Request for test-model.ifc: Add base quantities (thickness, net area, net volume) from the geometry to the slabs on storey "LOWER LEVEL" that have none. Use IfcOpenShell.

First a look at what the model holds.

```python
import ifcopenshell
import ifcopenshell.util.element
import ifcopenshell.util.unit

model = ifcopenshell.open("test-model.ifc")
print(model.schema)
for unit_type in ("LENGTHUNIT", "AREAUNIT", "VOLUMEUNIT"):
    print(unit_type, ifcopenshell.util.unit.calculate_unit_scale(model, unit_type))
storey = next(s for s in model.by_type("IfcBuildingStorey") if s.Name == "LOWER LEVEL")
slabs = [e for e in ifcopenshell.util.element.get_decomposition(storey) if e.is_a("IfcSlab")]
for e in sorted(slabs, key=lambda e: e.id()):
    print(e.id(), e.is_a(), e.Name, list(ifcopenshell.util.element.get_psets(e, qtos_only=True)), sep=" | ")
```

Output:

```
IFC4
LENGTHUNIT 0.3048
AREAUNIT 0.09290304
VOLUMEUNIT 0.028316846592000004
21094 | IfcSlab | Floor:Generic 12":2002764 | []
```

```python
import ifcopenshell
import ifcopenshell.api.pset
import ifcopenshell.geom
import ifcopenshell.util.element
import ifcopenshell.util.shape
import ifcopenshell.util.unit

model = ifcopenshell.open("test-model.ifc")
unit_scale = ifcopenshell.util.unit.calculate_unit_scale(model)
area_scale = ifcopenshell.util.unit.calculate_unit_scale(model, "AREAUNIT")
volume_scale = ifcopenshell.util.unit.calculate_unit_scale(model, "VOLUMEUNIT")
settings = ifcopenshell.geom.settings()

storey = next(s for s in model.by_type("IfcBuildingStorey") if s.Name == "LOWER LEVEL")
slabs = [e for e in ifcopenshell.util.element.get_decomposition(storey) if e.is_a("IfcSlab")]

for e in sorted(slabs, key=lambda e: e.id()):
    if ifcopenshell.util.element.get_psets(e, qtos_only=True, should_inherit=False):
        continue
    # Geometry comes back in metres, in the element's own axes.
    shape = ifcopenshell.geom.create_shape(settings, e)
    values = {
        "Width": ifcopenshell.util.shape.get_z(shape.geometry) / unit_scale,
        "NetArea": ifcopenshell.util.shape.get_footprint_area(shape.geometry) / area_scale,
        "NetVolume": ifcopenshell.util.shape.get_volume(shape.geometry) / volume_scale,
    }
    qto = ifcopenshell.api.pset.add_qto(model, product=e, name="Qto_SlabBaseQuantities")
    ifcopenshell.api.pset.edit_qto(model, qto=qto, properties=values)
    print(e.id(), {k: round(v, 3) for k, v in values.items()})

model.write("test-model_rev.ifc")
```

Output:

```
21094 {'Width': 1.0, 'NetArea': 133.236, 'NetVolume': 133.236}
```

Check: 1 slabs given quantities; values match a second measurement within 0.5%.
